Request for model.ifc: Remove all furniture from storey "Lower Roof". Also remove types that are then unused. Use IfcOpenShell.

First a look at what the model holds.

```python
import ifcopenshell
import ifcopenshell.util.element

model = ifcopenshell.open("model.ifc")
print(model.schema)
storey = next(s for s in model.by_type("IfcBuildingStorey") if s.Name == "Lower Roof")
furniture = [e for e in ifcopenshell.util.element.get_decomposition(storey) if e.is_a("IfcFurnishingElement")]
seen = {}
for e in furniture:
    element_type = ifcopenshell.util.element.get_type(e)
    name = element_type.Name if element_type not in (None, e) else None
    seen[name] = seen.get(name, 0) + 1
for name, count in sorted(seen.items(), key=str):
    print(count, "x", name)
```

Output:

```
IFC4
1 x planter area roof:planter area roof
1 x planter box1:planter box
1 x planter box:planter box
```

```python
import ifcopenshell
import ifcopenshell.api.root
import ifcopenshell.util.element

model = ifcopenshell.open("model.ifc")

storey = next(s for s in model.by_type("IfcBuildingStorey") if s.Name == "Lower Roof")
furniture = [e for e in ifcopenshell.util.element.get_decomposition(storey) if e.is_a("IfcFurnishingElement")]
types = {ifcopenshell.util.element.get_type(e) for e in furniture} - {None, *furniture}

for e in furniture:
    ifcopenshell.api.root.remove_product(model, product=e)
print(len(furniture), "removed")

unused = [t for t in types if not ifcopenshell.util.element.get_types(t)]
for t in unused:
    ifcopenshell.api.root.remove_product(model, product=t)
print(len(unused), "unused types removed")

model.write("model_updated.ifc")
```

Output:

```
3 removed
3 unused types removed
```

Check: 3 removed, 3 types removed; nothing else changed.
